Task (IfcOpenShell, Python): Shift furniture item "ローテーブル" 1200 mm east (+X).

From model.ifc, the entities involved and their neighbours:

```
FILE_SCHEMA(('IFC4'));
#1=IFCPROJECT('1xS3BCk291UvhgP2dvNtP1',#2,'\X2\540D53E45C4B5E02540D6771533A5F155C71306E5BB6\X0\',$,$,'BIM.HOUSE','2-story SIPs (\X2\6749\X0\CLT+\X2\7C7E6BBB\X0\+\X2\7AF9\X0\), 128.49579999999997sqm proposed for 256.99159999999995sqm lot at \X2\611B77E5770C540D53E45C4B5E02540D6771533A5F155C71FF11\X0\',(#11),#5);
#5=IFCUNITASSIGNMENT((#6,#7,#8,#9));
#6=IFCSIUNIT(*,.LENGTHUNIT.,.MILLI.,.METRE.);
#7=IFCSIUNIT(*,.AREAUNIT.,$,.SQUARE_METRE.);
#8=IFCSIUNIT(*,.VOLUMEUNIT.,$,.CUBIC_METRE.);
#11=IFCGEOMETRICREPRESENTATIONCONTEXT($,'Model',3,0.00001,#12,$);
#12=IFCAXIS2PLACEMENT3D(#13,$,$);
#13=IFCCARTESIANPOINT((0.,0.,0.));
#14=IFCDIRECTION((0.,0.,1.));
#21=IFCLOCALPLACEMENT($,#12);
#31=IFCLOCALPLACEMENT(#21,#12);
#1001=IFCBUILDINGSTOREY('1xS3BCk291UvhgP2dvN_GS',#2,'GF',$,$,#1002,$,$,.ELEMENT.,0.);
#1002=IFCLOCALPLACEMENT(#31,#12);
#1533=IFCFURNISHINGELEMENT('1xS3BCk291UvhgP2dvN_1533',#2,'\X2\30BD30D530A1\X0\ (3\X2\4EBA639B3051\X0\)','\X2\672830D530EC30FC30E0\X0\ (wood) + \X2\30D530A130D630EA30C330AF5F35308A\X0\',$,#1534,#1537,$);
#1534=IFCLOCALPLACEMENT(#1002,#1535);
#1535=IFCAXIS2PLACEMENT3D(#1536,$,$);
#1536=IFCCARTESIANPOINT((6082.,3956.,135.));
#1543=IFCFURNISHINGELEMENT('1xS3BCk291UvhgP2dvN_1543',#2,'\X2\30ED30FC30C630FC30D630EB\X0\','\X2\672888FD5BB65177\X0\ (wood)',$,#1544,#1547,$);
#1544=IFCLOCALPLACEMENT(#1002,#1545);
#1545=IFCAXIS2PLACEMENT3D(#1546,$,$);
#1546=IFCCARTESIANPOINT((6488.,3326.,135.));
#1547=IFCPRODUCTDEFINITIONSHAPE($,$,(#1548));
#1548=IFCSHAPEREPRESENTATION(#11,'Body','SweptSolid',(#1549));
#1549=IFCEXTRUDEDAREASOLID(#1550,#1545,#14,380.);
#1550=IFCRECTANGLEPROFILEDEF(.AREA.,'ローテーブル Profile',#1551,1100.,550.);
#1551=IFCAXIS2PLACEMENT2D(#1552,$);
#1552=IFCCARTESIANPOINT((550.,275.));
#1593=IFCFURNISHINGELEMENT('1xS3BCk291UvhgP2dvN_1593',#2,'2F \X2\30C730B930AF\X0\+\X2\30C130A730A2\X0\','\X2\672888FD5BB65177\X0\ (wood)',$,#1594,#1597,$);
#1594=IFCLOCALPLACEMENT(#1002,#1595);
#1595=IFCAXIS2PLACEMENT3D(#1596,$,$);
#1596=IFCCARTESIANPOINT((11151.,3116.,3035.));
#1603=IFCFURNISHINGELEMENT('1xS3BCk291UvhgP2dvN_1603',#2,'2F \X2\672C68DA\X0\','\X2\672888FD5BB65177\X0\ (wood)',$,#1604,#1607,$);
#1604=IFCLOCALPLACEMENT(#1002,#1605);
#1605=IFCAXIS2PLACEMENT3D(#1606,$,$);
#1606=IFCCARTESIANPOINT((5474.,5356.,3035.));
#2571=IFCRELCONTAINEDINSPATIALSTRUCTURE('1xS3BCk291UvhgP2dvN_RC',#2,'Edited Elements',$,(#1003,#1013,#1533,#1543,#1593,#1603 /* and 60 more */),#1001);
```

```python
import ifcopenshell
import ifcopenshell.api.geometry
import ifcopenshell.util.placement
import ifcopenshell.util.unit

model = ifcopenshell.open("model.ifc")
unit_scale = ifcopenshell.util.unit.calculate_unit_scale(model)

item = model.by_id(1543)
matrix = ifcopenshell.util.placement.get_local_placement(item.ObjectPlacement)
matrix[0, 3] += 1.2 / unit_scale
ifcopenshell.api.geometry.edit_object_placement(model, product=item, matrix=matrix, is_si=False)

print(ifcopenshell.util.placement.get_local_placement(item.ObjectPlacement).round(3) + 0.0)

model.write("model_edited.ifc")
```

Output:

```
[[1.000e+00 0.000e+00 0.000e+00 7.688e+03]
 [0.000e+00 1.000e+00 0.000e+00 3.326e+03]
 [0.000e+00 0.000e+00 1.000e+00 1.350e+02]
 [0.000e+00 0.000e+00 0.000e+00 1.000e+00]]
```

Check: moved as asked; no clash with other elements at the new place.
